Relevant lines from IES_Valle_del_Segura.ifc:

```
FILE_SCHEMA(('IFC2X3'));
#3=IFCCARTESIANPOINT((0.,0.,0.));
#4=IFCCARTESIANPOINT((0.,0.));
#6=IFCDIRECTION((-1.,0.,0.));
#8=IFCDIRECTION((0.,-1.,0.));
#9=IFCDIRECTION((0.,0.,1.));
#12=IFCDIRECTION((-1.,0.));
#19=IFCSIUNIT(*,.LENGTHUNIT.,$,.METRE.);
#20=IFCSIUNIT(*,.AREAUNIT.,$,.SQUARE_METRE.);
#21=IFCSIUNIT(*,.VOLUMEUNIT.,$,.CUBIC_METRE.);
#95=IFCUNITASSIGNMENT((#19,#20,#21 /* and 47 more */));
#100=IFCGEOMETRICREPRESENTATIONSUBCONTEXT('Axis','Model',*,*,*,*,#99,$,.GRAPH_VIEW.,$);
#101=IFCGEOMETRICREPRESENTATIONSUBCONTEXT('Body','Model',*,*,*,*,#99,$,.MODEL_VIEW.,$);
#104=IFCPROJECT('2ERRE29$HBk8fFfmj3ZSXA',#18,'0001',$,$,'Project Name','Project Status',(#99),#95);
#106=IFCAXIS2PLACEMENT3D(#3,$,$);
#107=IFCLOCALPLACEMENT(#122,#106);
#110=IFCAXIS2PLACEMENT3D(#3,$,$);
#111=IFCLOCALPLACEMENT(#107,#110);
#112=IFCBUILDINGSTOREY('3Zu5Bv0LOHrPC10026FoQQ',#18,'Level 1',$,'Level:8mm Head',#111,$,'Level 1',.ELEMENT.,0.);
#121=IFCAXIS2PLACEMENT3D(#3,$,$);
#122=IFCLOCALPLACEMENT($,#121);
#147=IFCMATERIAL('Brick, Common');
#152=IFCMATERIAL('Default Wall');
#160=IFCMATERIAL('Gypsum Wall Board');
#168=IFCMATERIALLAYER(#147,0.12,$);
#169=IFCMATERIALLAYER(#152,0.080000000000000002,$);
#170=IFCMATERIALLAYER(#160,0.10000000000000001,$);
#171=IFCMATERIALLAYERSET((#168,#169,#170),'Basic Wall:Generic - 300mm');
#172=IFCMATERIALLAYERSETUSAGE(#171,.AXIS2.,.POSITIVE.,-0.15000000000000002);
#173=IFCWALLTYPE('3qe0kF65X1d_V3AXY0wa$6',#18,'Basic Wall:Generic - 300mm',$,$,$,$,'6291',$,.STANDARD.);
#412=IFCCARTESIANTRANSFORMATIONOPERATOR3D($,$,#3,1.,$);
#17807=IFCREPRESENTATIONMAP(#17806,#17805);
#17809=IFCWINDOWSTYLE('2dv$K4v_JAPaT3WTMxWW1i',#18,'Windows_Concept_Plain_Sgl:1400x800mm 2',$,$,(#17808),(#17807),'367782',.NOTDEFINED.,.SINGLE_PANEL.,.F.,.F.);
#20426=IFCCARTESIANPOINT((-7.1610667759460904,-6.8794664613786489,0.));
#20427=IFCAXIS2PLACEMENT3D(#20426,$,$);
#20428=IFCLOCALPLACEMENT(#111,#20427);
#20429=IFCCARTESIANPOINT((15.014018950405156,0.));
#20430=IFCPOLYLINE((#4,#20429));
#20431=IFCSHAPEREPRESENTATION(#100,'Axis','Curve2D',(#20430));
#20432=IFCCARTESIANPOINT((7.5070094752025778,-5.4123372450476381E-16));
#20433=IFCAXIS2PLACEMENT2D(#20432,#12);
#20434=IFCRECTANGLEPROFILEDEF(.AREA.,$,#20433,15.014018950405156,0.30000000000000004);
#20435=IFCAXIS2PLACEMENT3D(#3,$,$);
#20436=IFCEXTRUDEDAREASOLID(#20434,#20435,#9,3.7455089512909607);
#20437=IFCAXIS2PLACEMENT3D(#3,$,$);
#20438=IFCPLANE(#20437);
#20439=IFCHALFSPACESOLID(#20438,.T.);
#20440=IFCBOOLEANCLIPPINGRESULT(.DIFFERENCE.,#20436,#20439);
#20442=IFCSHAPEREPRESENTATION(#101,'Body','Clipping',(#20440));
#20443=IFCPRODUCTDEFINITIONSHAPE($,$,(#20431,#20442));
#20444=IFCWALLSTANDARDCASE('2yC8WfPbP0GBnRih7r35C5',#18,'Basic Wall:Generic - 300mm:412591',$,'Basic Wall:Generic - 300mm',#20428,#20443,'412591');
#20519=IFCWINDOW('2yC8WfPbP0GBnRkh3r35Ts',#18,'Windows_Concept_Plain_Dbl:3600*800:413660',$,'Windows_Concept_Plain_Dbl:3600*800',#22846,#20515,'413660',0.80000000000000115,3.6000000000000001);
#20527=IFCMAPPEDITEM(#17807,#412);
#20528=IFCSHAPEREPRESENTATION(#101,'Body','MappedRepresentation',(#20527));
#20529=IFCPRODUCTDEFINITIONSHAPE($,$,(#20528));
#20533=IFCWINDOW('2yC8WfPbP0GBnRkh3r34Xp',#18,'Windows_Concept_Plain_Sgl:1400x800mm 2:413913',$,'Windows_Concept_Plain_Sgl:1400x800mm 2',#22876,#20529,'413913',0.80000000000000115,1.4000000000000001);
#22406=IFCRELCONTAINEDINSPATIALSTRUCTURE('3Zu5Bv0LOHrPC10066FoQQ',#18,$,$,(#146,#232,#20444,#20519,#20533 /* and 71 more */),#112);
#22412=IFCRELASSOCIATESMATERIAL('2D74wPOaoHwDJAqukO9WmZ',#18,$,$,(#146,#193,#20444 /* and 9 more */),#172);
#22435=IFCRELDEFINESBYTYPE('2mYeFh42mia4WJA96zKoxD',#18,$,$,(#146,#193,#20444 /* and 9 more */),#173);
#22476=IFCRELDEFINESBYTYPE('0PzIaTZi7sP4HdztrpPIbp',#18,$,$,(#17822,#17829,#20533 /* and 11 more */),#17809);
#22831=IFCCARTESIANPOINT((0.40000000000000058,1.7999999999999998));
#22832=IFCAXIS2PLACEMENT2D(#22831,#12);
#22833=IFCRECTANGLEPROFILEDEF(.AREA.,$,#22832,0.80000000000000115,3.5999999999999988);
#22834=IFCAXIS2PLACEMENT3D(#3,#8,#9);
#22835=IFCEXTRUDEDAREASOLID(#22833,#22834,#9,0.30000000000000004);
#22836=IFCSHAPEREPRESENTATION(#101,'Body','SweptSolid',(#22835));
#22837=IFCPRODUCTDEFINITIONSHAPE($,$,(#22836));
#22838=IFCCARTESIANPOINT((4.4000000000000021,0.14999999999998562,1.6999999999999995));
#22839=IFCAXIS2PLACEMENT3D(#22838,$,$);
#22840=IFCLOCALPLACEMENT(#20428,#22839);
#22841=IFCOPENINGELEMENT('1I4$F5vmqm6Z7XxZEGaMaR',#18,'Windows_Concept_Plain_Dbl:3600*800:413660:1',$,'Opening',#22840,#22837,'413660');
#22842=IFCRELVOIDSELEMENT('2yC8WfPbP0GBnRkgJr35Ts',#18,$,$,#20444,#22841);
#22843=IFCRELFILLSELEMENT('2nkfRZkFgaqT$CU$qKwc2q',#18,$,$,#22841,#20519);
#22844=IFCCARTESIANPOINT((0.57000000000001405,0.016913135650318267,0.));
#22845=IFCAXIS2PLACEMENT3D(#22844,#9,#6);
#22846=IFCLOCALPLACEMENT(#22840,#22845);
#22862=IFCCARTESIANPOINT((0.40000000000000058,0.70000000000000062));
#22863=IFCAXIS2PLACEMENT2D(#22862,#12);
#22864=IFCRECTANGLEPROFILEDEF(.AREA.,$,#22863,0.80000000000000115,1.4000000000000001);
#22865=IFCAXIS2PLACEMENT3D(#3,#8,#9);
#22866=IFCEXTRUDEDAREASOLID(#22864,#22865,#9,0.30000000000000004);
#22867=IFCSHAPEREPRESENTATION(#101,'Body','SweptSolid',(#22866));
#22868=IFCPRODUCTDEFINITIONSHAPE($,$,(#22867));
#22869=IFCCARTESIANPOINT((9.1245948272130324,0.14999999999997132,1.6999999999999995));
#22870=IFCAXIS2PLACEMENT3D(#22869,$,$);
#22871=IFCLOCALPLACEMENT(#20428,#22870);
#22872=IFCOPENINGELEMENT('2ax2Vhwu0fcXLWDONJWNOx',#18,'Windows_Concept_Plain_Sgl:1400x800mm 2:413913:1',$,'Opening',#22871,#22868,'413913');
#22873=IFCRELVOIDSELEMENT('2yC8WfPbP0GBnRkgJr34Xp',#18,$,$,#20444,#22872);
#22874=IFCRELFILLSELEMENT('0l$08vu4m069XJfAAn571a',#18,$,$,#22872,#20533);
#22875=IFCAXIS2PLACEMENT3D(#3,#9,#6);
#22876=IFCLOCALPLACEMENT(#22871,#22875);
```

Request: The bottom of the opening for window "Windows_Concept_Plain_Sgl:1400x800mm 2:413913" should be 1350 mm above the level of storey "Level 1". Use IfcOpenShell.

```python
import numpy as np
import ifcopenshell
import ifcopenshell.api.geometry
import ifcopenshell.geom
import ifcopenshell.util.element
import ifcopenshell.util.placement
import ifcopenshell.util.shape
import ifcopenshell.util.unit

model = ifcopenshell.open("IES_Valle_del_Segura.ifc")
unit_scale = ifcopenshell.util.unit.calculate_unit_scale(model)

window = model.by_id(20533)
opening = window.FillsVoids[0].RelatingOpeningElement
storey = ifcopenshell.util.element.get_container(window, ifc_class="IfcBuildingStorey")
level = ifcopenshell.util.placement.get_local_placement(storey.ObjectPlacement)[2, 3]

# The opening's origin need not be at the sill, so measure its lowest point.
shape = ifcopenshell.geom.create_shape(ifcopenshell.geom.settings(), opening)
bottom = ifcopenshell.util.shape.get_shape_bottom_elevation(shape, shape.geometry) / unit_scale
dz = level + 1.35 - bottom

shift = np.array([0.0, 0.0, dz])
# The window is placed relative to its opening, so it follows when the opening moves.
matrix = ifcopenshell.util.placement.get_local_placement(opening.ObjectPlacement)
matrix[:3, 3] += shift
ifcopenshell.api.geometry.edit_object_placement(
    model, product=opening, matrix=matrix, is_si=False, should_transform_children=True
)

print(f"moved by {dz * unit_scale:+.3f} m")

model.write("IES_Valle_del_Segura_edited.ifc")
```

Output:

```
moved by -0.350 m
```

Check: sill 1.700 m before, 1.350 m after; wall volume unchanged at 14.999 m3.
